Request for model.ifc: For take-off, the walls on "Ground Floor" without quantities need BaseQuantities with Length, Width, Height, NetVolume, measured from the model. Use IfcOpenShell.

First a look at what the model holds.

```python
import ifcopenshell
import ifcopenshell.util.element
import ifcopenshell.util.unit

model = ifcopenshell.open("model.ifc")
print(model.schema)
for unit_type in ("LENGTHUNIT", "AREAUNIT", "VOLUMEUNIT"):
    print(unit_type, ifcopenshell.util.unit.calculate_unit_scale(model, unit_type))
storey = next(s for s in model.by_type("IfcBuildingStorey") if s.Name == "Ground Floor")
walls = [e for e in ifcopenshell.util.element.get_decomposition(storey) if e.is_a("IfcWall")]
for e in sorted(walls, key=lambda e: e.id()):
    print(e.id(), e.is_a(), e.Name, list(ifcopenshell.util.element.get_psets(e, qtos_only=True)), sep=" | ")
```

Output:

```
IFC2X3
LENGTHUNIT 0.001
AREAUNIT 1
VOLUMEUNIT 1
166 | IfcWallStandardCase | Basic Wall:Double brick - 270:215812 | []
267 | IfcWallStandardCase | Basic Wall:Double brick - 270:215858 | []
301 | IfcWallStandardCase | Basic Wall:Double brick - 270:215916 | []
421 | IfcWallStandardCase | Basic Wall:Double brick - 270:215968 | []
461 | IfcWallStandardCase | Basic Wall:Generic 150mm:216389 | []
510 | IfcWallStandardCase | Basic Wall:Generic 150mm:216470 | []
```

```python
import ifcopenshell
import ifcopenshell.api.pset
import ifcopenshell.geom
import ifcopenshell.util.element
import ifcopenshell.util.shape
import ifcopenshell.util.unit

model = ifcopenshell.open("model.ifc")
unit_scale = ifcopenshell.util.unit.calculate_unit_scale(model)
volume_scale = ifcopenshell.util.unit.calculate_unit_scale(model, "VOLUMEUNIT")
settings = ifcopenshell.geom.settings()

storey = next(s for s in model.by_type("IfcBuildingStorey") if s.Name == "Ground Floor")
walls = [e for e in ifcopenshell.util.element.get_decomposition(storey) if e.is_a("IfcWall")]

for e in sorted(walls, key=lambda e: e.id()):
    if ifcopenshell.util.element.get_psets(e, qtos_only=True, should_inherit=False):
        continue
    # Geometry comes back in metres, in the element's own axes.
    shape = ifcopenshell.geom.create_shape(settings, e)
    values = {
        "Length": ifcopenshell.util.shape.get_x(shape.geometry) / unit_scale,
        "Width": ifcopenshell.util.shape.get_y(shape.geometry) / unit_scale,
        "Height": ifcopenshell.util.shape.get_z(shape.geometry) / unit_scale,
        "NetVolume": ifcopenshell.util.shape.get_volume(shape.geometry) / volume_scale,
    }
    qto = ifcopenshell.api.pset.add_qto(model, product=e, name="BaseQuantities")
    ifcopenshell.api.pset.edit_qto(model, qto=qto, properties=values)
    print(e.id(), {k: round(v, 3) for k, v in values.items()})

model.write("model_updated.ifc")
```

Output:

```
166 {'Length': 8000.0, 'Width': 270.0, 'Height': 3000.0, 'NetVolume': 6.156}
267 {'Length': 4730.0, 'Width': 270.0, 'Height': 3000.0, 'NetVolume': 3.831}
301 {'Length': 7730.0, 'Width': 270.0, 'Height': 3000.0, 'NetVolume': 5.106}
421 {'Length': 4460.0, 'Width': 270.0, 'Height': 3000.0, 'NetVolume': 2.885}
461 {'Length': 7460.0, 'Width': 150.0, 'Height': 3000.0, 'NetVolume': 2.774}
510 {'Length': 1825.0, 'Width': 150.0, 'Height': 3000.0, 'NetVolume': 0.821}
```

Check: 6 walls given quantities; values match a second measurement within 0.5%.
